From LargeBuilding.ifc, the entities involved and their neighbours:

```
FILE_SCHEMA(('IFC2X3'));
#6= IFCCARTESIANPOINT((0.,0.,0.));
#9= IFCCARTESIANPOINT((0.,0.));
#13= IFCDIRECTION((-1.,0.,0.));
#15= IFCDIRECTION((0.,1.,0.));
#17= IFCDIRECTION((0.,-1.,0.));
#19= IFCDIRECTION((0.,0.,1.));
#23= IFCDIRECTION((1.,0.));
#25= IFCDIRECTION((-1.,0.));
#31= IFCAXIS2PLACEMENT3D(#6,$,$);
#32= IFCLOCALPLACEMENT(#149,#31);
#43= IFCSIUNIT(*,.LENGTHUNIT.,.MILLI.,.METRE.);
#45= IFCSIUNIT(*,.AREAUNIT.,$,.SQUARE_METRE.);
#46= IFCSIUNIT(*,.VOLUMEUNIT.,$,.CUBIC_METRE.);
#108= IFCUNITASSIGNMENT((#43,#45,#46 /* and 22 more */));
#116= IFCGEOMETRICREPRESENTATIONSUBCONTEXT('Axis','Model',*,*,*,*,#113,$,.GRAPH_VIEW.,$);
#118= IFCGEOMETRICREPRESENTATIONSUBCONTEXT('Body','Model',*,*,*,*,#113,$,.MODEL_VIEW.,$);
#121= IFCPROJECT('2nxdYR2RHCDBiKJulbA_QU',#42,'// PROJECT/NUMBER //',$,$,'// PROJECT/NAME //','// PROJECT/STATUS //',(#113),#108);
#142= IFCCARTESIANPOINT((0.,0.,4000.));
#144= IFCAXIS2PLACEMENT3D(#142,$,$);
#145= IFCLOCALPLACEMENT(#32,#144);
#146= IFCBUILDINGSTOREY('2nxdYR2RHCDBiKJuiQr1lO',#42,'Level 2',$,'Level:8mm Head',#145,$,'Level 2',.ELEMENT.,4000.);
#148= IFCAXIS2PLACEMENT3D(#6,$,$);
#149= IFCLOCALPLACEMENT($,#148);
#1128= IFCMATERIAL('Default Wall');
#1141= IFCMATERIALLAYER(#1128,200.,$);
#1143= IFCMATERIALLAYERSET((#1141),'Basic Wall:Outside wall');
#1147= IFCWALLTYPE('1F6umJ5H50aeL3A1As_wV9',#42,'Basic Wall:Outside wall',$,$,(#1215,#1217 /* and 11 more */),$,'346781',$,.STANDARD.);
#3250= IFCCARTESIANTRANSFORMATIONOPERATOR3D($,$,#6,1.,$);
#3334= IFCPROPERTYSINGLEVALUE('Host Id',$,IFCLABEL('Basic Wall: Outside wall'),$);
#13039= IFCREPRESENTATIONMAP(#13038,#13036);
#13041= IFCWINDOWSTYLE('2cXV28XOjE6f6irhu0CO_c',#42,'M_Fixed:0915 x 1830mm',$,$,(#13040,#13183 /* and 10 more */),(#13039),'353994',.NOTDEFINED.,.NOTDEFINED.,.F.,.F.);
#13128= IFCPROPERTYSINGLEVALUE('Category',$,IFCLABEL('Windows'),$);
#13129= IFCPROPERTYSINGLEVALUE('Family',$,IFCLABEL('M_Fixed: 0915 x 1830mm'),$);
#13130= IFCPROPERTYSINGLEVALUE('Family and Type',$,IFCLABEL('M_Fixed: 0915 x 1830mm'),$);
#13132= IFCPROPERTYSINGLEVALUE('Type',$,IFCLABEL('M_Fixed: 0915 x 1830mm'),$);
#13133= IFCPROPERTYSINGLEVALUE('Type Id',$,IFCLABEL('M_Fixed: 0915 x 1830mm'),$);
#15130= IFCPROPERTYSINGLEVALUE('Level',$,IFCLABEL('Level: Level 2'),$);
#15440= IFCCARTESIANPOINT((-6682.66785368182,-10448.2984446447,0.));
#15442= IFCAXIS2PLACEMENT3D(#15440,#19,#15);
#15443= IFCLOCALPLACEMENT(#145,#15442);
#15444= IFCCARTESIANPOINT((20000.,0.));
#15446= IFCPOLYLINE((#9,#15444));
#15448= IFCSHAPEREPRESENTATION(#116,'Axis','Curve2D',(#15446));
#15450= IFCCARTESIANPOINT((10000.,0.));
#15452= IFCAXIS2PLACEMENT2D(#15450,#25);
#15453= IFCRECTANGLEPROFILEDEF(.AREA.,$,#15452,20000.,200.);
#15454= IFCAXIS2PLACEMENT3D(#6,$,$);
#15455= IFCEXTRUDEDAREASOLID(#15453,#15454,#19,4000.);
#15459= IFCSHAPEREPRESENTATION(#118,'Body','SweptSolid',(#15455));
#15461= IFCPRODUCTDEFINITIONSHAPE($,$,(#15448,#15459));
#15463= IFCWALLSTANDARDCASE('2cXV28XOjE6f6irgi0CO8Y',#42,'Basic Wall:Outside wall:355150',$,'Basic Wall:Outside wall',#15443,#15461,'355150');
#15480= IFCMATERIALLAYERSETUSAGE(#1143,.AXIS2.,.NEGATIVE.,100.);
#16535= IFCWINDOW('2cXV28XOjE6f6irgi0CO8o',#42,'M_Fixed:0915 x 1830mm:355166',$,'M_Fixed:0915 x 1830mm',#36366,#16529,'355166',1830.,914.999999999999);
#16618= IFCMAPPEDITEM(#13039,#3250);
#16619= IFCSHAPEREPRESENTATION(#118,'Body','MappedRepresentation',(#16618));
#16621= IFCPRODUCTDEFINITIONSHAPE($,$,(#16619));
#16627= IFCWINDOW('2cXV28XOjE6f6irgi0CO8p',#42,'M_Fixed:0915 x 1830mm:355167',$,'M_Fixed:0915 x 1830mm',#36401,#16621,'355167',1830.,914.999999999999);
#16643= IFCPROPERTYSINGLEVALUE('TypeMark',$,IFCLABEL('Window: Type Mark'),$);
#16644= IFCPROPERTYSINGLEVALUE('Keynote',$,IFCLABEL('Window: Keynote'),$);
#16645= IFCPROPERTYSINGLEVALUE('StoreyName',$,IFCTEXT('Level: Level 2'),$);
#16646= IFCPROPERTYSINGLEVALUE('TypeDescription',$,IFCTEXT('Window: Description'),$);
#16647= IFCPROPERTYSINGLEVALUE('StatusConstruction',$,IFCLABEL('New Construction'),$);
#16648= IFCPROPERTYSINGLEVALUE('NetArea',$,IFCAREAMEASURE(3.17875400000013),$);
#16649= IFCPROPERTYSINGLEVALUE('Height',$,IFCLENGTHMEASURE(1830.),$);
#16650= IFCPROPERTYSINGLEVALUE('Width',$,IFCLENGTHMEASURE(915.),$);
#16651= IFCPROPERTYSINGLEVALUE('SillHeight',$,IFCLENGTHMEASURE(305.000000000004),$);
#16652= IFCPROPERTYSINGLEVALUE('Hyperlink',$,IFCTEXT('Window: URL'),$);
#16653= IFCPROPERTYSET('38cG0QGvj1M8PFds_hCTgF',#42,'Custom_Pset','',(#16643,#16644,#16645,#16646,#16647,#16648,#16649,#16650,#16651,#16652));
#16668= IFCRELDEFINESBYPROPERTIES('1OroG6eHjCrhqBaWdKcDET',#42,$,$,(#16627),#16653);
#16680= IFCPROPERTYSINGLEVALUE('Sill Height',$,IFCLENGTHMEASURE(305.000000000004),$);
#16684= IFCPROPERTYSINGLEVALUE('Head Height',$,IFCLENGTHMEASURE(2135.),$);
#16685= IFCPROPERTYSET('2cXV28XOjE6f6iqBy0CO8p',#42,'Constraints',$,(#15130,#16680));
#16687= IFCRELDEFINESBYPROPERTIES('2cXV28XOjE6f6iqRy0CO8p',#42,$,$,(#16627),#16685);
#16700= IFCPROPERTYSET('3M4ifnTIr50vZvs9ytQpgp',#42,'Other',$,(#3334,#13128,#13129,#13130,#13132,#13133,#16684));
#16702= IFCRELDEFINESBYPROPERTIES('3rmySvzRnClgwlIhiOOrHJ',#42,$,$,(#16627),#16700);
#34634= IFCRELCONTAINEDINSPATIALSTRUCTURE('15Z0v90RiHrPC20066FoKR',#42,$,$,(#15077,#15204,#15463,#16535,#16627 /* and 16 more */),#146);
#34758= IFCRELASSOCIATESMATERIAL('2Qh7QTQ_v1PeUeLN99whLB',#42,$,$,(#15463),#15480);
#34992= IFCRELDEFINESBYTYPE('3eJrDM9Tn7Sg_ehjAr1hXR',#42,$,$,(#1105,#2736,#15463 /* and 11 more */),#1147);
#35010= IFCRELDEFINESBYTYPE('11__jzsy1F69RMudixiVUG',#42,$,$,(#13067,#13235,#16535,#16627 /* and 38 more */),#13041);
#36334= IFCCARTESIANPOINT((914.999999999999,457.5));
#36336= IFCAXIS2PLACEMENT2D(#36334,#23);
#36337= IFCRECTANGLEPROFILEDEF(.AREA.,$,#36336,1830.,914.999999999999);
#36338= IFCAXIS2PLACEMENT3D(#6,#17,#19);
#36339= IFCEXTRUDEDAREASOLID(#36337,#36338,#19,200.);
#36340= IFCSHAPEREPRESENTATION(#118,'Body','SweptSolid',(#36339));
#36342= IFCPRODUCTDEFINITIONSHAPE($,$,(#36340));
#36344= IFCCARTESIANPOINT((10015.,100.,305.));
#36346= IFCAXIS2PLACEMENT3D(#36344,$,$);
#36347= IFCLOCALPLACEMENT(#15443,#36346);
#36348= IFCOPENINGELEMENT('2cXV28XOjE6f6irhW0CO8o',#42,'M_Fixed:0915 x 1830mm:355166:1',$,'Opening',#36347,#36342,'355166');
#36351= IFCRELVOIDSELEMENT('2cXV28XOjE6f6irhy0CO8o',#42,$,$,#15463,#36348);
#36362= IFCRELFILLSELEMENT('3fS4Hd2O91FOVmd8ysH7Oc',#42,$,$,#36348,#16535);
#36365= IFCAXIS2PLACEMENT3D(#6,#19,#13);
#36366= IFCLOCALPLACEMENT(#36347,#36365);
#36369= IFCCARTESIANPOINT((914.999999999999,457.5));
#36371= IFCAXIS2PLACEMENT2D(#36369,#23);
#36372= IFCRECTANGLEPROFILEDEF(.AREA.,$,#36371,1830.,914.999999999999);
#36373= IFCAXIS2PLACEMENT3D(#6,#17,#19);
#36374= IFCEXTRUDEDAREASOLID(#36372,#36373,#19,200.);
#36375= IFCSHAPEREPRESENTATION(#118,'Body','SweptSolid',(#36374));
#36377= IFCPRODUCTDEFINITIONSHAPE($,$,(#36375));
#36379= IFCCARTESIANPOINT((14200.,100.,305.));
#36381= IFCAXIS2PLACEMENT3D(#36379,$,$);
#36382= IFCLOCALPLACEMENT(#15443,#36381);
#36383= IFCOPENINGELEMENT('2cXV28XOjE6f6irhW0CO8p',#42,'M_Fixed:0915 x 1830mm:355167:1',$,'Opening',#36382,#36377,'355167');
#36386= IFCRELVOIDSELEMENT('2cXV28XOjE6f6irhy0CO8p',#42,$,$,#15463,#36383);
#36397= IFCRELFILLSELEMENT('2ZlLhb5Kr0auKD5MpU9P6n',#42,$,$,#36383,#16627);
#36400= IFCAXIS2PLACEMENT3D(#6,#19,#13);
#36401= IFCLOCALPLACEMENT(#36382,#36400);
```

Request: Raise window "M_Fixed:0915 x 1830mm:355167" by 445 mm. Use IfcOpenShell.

```python
import numpy as np
import ifcopenshell
import ifcopenshell.api.geometry
import ifcopenshell.api.pset
import ifcopenshell.util.element
import ifcopenshell.util.placement
import ifcopenshell.util.unit

model = ifcopenshell.open("LargeBuilding.ifc")
unit_scale = ifcopenshell.util.unit.calculate_unit_scale(model)

window = model.by_guid("2cXV28XOjE6f6irgi0CO8p")
opening = window.FillsVoids[0].RelatingOpeningElement
dz = 445.0

shift = np.array([0.0, 0.0, dz])
# The window is placed relative to its opening, so it follows when the opening moves.
matrix = ifcopenshell.util.placement.get_local_placement(opening.ObjectPlacement)
matrix[:3, 3] += shift
ifcopenshell.api.geometry.edit_object_placement(
    model, product=opening, matrix=matrix, is_si=False, should_transform_children=True
)

# Keep the stored heights in step.
pset = model.by_id(ifcopenshell.util.element.get_pset(window, "Custom_Pset", should_inherit=False)["id"])
ifcopenshell.api.pset.edit_pset(model, pset=pset, properties={
    "SillHeight": model.create_entity("IfcLengthMeasure", ifcopenshell.util.element.get_pset(window, "Constraints", "Sill Height") + dz),
})
pset = model.by_id(ifcopenshell.util.element.get_pset(window, "Constraints", should_inherit=False)["id"])
ifcopenshell.api.pset.edit_pset(model, pset=pset, properties={
    "Sill Height": model.create_entity("IfcLengthMeasure", ifcopenshell.util.element.get_pset(window, "Constraints", "Sill Height") + dz),
})
pset = model.by_id(ifcopenshell.util.element.get_pset(window, "Other", should_inherit=False)["id"])
ifcopenshell.api.pset.edit_pset(model, pset=pset, properties={
    "Head Height": model.create_entity("IfcLengthMeasure", ifcopenshell.util.element.get_pset(window, "Other", "Head Height") + dz),
})

print(f"moved by {dz * unit_scale:+.3f} m")

model.write("LargeBuilding_edited.ifc")
```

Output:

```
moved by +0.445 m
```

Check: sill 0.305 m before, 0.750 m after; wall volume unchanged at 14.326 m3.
